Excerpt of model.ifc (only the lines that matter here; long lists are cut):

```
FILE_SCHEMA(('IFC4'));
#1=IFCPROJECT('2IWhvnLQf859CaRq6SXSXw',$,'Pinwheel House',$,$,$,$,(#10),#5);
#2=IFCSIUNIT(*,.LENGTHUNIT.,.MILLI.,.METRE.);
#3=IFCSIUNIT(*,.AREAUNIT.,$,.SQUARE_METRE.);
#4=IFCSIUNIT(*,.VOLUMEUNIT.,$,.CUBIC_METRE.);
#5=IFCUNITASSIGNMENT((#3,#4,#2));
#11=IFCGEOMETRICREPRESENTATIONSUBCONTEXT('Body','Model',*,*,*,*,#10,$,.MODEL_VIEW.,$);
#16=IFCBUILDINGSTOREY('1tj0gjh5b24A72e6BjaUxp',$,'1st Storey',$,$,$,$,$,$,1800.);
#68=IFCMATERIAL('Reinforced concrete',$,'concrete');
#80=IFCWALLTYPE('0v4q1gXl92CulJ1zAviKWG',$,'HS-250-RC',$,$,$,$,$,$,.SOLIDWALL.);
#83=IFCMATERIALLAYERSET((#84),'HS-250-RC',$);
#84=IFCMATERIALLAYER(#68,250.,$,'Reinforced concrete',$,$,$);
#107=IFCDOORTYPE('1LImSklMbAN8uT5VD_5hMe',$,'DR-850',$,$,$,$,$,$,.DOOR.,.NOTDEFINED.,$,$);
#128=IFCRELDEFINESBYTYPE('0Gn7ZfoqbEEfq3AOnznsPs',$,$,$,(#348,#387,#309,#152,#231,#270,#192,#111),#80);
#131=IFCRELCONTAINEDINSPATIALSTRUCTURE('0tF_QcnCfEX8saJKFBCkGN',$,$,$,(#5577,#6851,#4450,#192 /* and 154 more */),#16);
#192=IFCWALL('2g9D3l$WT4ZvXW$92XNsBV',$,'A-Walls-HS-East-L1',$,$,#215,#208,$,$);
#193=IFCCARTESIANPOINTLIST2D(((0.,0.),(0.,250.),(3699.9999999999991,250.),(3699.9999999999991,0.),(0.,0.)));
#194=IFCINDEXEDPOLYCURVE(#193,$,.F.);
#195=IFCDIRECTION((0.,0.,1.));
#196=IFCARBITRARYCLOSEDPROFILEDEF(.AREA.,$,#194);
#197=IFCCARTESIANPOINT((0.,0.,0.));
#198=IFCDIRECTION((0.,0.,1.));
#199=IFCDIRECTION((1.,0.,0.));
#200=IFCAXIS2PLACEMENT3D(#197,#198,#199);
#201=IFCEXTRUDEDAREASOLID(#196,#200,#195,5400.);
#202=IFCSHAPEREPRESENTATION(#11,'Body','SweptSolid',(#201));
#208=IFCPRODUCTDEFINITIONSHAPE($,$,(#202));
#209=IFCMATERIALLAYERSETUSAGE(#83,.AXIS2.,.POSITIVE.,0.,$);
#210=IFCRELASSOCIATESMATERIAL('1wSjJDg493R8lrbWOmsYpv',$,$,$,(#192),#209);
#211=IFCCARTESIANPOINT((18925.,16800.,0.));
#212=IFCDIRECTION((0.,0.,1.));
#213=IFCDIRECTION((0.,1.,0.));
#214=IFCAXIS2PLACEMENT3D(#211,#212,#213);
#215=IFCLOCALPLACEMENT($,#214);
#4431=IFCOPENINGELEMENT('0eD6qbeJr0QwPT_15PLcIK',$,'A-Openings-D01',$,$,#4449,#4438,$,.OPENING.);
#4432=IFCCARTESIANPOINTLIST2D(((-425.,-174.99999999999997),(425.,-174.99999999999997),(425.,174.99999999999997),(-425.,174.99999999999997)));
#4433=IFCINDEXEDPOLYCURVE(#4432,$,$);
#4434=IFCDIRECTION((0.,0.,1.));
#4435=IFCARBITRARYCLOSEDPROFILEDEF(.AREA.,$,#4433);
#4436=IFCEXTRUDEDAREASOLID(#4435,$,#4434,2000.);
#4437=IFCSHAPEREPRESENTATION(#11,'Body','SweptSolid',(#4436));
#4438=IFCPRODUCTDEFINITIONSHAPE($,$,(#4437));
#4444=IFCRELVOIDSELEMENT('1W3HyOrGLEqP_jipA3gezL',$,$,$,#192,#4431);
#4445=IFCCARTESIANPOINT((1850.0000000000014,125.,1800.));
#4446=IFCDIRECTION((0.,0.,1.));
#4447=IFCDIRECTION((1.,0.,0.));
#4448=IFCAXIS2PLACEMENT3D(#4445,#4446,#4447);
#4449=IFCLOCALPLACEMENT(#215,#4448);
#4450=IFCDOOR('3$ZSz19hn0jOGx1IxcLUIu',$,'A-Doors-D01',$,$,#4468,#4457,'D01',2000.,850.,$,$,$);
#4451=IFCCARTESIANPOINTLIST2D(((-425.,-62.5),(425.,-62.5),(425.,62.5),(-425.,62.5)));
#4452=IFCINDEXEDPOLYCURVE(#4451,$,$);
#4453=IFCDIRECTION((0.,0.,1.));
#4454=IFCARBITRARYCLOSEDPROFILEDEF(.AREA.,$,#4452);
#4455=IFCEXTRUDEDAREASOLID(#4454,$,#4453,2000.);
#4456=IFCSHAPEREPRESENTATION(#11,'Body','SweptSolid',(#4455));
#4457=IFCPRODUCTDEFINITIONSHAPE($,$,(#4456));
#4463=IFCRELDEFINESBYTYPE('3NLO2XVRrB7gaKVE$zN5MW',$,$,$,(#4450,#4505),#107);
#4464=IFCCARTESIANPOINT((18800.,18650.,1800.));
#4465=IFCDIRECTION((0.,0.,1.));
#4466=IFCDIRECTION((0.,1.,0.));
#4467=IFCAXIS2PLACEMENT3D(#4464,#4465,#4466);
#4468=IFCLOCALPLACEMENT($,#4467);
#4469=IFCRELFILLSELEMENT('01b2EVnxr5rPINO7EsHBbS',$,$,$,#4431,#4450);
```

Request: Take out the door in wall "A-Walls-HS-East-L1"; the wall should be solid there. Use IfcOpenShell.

```python
import ifcopenshell
import ifcopenshell.api.feature
import ifcopenshell.api.root
import ifcopenshell.geom
import ifcopenshell.util.shape

model = ifcopenshell.open("model.ifc")
settings = ifcopenshell.geom.settings()


def volume(element):
    """Net volume in cubic metres, openings subtracted."""
    shape = ifcopenshell.geom.create_shape(settings, element)
    return ifcopenshell.util.shape.get_volume(shape.geometry)


door = model.by_guid("3$ZSz19hn0jOGx1IxcLUIu")
opening = door.FillsVoids[0].RelatingOpeningElement
wall = opening.VoidsElements[0].RelatingBuildingElement
before = volume(wall)

ifcopenshell.api.root.remove_product(model, product=door)
ifcopenshell.api.feature.remove_feature(model, feature=opening)

after = volume(wall)

print(f"wall volume {before:.3f} -> {after:.3f} m3")

model.write("model_edited.ifc")
```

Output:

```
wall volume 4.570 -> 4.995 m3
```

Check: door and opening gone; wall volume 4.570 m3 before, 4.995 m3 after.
